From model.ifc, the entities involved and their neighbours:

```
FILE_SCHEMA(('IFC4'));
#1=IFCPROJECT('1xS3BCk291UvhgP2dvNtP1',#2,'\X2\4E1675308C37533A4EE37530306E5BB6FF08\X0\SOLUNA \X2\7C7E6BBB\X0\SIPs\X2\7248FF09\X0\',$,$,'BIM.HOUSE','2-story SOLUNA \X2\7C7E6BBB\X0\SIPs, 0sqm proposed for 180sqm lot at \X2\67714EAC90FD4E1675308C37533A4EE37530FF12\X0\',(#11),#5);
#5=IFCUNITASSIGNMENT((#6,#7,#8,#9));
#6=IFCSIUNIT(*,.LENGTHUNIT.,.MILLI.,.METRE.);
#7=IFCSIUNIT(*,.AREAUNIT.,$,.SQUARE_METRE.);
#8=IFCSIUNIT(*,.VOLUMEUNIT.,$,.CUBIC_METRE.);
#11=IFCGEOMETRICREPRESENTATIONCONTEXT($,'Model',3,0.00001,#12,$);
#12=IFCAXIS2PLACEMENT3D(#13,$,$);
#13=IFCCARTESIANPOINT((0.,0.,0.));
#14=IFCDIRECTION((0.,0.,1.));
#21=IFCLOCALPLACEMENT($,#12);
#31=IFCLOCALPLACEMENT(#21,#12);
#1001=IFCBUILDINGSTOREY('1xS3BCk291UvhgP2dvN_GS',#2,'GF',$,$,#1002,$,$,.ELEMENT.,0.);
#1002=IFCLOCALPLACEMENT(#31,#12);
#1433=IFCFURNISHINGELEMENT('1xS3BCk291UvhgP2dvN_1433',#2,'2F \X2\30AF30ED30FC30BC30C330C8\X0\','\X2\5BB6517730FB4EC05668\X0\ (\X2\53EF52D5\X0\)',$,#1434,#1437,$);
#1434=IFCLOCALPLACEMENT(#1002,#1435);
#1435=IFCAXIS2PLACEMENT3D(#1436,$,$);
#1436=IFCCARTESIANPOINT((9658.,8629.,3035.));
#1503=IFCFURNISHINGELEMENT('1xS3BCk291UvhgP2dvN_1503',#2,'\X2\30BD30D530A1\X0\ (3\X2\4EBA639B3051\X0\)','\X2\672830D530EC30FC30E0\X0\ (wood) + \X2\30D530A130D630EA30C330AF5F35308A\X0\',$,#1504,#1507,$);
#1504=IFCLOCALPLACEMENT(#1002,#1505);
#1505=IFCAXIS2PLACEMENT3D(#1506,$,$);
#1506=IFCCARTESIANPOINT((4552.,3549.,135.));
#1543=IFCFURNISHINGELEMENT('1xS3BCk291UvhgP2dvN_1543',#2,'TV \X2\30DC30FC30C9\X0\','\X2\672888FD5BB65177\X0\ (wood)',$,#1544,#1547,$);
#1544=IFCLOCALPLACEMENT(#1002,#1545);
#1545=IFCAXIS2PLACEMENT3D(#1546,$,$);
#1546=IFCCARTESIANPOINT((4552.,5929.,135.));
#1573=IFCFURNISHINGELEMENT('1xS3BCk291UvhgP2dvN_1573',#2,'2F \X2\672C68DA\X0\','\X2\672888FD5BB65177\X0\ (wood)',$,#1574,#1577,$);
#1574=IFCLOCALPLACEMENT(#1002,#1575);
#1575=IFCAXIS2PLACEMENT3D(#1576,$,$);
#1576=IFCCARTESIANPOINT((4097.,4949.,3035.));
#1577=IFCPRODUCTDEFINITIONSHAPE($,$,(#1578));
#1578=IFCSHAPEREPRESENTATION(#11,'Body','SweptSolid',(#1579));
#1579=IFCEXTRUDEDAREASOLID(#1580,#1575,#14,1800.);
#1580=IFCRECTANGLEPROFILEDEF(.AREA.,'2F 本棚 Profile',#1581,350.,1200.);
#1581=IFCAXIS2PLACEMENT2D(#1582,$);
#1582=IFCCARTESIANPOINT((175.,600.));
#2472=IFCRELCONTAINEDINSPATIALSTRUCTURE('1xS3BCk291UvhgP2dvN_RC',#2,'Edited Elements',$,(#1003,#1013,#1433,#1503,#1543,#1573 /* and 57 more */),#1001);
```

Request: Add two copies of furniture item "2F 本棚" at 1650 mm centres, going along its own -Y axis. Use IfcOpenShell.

```python
import ifcopenshell
import ifcopenshell.api.geometry
import ifcopenshell.api.root
import ifcopenshell.util.element
import ifcopenshell.util.placement

model = ifcopenshell.open("model.ifc")


def reuse_history(source, copy):
    """copy_class also copies each property set's owner history, people and application; keep the originals."""
    for rel in copy.IsDefinedBy:
        if rel.is_a("IfcRelDefinesByProperties") and (history := rel.RelatingPropertyDefinition.OwnerHistory):
            rel.RelatingPropertyDefinition.OwnerHistory = source.OwnerHistory
            ifcopenshell.util.element.remove_deep2(model, history)


source = model.by_guid("1xS3BCk291UvhgP2dvN_1573")
base = ifcopenshell.util.placement.get_local_placement(source.ObjectPlacement)
step = -base[:3, 1] * 1650.0

for i in range(1, 3):
    copy = ifcopenshell.api.root.copy_class(model, product=source)
    copy.Representation = ifcopenshell.util.element.copy_deep(
        model, source.Representation, exclude=["IfcGeometricRepresentationContext", "IfcRepresentationMap"]
    )
    reuse_history(source, copy)
    matrix = base.copy()
    matrix[:3, 3] += i * step
    print("added at", matrix[:3, 3].round(3) + 0.0)
    ifcopenshell.api.geometry.edit_object_placement(model, product=copy, matrix=matrix, is_si=False)

model.write("model_edited.ifc")
```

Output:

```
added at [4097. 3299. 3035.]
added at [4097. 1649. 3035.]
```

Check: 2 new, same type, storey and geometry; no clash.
